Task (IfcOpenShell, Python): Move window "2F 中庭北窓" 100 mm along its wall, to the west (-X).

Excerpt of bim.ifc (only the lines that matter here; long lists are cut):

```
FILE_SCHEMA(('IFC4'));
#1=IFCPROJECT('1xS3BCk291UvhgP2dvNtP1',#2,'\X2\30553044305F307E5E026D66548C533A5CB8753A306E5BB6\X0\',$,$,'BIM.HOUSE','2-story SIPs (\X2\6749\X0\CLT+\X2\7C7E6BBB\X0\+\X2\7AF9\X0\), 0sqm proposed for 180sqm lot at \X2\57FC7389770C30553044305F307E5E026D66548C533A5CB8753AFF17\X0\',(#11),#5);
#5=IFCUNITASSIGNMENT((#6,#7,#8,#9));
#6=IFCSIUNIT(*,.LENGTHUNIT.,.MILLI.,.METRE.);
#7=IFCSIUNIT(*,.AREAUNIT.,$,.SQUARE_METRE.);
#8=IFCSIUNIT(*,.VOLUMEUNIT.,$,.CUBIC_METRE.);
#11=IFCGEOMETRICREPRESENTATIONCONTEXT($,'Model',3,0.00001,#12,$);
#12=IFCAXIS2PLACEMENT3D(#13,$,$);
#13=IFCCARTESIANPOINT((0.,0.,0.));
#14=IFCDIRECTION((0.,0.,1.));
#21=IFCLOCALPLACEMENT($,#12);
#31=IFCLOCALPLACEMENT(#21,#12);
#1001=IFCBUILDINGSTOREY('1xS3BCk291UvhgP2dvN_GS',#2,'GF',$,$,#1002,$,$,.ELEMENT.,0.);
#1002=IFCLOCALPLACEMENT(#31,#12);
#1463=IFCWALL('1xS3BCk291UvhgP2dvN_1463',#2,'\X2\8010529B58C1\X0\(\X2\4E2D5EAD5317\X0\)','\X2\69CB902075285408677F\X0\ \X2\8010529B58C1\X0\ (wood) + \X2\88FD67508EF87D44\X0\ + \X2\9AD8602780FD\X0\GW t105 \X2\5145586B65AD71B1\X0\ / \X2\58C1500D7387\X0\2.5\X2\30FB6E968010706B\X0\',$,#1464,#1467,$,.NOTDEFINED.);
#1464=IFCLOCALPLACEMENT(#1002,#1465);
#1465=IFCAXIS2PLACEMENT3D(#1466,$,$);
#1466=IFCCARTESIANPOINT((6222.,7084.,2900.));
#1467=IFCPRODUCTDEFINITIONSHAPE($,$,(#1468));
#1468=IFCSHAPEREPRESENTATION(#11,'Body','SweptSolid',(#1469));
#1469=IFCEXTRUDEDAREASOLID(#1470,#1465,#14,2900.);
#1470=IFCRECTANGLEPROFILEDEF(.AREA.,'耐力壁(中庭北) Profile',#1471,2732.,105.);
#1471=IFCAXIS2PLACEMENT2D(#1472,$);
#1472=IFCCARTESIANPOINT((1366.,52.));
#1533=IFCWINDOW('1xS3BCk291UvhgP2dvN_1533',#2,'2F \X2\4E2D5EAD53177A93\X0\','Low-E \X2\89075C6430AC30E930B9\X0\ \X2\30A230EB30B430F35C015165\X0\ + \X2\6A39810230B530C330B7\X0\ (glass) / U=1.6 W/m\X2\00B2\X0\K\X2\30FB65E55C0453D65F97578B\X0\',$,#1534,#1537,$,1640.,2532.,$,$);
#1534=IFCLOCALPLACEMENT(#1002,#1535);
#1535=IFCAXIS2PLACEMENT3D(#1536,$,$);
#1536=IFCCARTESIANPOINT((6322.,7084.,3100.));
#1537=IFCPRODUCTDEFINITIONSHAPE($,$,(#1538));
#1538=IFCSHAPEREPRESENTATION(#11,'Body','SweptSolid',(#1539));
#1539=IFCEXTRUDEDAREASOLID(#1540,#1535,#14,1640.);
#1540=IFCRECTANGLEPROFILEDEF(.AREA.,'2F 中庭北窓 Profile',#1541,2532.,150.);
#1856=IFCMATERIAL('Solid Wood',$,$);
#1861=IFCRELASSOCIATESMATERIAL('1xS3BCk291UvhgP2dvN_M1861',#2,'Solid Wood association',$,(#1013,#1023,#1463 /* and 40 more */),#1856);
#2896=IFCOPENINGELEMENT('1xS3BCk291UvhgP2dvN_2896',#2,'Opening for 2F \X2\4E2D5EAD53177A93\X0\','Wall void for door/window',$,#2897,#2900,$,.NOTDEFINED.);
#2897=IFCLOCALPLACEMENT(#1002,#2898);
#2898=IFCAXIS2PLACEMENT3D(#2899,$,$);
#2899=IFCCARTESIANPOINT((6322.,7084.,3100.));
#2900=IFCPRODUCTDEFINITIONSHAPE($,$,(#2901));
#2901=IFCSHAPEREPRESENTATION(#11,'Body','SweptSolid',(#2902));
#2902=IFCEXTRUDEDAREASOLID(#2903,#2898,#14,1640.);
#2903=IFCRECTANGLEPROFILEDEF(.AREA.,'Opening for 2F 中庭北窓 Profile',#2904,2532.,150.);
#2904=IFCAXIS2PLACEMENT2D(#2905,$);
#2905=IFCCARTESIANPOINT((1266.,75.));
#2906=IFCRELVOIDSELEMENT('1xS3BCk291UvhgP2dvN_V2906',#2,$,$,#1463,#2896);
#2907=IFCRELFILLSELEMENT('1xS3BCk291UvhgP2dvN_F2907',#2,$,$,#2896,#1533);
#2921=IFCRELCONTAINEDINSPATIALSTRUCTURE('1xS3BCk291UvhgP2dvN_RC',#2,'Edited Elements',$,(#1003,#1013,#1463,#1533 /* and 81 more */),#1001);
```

```python
import ifcopenshell
import ifcopenshell.api.geometry
import ifcopenshell.util.placement
import ifcopenshell.util.unit

model = ifcopenshell.open("bim.ifc")
unit_scale = ifcopenshell.util.unit.calculate_unit_scale(model)

window = model.by_guid("1xS3BCk291UvhgP2dvN_1533")
opening = window.FillsVoids[0].RelatingOpeningElement
wall = opening.VoidsElements[0].RelatingBuildingElement

wall_matrix = ifcopenshell.util.placement.get_local_placement(wall.ObjectPlacement)
shift = wall_matrix[:3, 0] * -0.1 / unit_scale
before = ifcopenshell.util.placement.get_local_placement(window.ObjectPlacement)[:3, 3].copy()

# The window is not placed relative to its opening, so move both.
for product in (opening, window):
    matrix = ifcopenshell.util.placement.get_local_placement(product.ObjectPlacement)
    matrix[:3, 3] += shift
    ifcopenshell.api.geometry.edit_object_placement(model, product=product, matrix=matrix, is_si=False)

after = ifcopenshell.util.placement.get_local_placement(window.ObjectPlacement)[:3, 3]
print("window moved by", (after - before).round(3) + 0.0)

model.write("bim-out.ifc")
```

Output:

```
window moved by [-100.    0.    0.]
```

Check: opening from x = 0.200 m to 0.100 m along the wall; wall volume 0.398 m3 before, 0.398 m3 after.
